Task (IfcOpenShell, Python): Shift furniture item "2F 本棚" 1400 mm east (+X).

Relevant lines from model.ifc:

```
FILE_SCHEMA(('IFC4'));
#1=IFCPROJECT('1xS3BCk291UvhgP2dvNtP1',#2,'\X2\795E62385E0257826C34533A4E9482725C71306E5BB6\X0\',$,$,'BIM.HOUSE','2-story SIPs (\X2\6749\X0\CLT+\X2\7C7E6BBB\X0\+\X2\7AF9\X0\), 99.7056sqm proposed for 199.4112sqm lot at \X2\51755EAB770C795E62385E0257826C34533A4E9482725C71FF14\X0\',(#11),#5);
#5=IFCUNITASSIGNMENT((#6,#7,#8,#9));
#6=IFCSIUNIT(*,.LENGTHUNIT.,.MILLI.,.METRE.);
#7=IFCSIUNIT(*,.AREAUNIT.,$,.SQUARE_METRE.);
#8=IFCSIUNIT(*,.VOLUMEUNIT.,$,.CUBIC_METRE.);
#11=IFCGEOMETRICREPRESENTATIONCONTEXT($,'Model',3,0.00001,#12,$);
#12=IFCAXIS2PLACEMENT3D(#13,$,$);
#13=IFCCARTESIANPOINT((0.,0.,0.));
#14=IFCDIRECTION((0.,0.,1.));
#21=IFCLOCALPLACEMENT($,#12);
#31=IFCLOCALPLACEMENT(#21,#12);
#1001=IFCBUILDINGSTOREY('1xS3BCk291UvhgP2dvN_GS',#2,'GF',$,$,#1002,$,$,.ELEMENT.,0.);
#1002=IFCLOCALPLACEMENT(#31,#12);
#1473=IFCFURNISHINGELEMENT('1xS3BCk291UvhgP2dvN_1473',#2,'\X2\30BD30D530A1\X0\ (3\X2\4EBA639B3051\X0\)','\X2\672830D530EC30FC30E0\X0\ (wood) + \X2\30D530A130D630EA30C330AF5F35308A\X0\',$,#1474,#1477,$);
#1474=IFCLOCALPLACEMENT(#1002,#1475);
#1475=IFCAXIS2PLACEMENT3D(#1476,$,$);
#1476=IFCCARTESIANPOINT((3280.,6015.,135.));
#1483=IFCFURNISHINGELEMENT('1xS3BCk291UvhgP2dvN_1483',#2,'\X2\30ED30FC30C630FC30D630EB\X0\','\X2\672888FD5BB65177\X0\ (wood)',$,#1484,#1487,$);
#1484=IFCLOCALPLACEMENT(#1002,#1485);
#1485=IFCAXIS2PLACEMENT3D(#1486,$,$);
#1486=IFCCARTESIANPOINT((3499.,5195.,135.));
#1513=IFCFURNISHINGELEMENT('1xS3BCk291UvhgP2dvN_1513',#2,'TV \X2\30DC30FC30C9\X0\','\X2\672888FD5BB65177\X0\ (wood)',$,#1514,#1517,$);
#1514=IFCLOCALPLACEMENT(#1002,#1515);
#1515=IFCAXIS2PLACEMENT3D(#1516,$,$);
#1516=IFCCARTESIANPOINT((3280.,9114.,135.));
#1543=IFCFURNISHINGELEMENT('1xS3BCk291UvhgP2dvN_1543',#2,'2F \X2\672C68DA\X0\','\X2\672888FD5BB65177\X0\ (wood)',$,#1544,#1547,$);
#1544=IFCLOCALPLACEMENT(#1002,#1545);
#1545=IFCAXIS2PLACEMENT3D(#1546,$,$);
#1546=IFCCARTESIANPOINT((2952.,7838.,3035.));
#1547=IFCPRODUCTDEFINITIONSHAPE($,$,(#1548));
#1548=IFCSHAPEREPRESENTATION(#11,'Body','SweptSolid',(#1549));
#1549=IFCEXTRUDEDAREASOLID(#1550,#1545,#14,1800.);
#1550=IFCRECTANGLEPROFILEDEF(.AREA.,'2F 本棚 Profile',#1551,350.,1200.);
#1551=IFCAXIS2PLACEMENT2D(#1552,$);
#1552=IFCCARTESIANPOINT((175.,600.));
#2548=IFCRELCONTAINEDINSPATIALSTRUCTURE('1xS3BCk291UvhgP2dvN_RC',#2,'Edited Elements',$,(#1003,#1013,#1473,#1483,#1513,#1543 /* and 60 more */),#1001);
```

```python
import ifcopenshell
import ifcopenshell.api.geometry
import ifcopenshell.util.placement
import ifcopenshell.util.unit

model = ifcopenshell.open("model.ifc")
unit_scale = ifcopenshell.util.unit.calculate_unit_scale(model)

item = model.by_guid("1xS3BCk291UvhgP2dvN_1543")
matrix = ifcopenshell.util.placement.get_local_placement(item.ObjectPlacement)
matrix[0, 3] += 1.4 / unit_scale
ifcopenshell.api.geometry.edit_object_placement(model, product=item, matrix=matrix, is_si=False)

print(ifcopenshell.util.placement.get_local_placement(item.ObjectPlacement).round(3) + 0.0)

model.write("model_edited.ifc")
```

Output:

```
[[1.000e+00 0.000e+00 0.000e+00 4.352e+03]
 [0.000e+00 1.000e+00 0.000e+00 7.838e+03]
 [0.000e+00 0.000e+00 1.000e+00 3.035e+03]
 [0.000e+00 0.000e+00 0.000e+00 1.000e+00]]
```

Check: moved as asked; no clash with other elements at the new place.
